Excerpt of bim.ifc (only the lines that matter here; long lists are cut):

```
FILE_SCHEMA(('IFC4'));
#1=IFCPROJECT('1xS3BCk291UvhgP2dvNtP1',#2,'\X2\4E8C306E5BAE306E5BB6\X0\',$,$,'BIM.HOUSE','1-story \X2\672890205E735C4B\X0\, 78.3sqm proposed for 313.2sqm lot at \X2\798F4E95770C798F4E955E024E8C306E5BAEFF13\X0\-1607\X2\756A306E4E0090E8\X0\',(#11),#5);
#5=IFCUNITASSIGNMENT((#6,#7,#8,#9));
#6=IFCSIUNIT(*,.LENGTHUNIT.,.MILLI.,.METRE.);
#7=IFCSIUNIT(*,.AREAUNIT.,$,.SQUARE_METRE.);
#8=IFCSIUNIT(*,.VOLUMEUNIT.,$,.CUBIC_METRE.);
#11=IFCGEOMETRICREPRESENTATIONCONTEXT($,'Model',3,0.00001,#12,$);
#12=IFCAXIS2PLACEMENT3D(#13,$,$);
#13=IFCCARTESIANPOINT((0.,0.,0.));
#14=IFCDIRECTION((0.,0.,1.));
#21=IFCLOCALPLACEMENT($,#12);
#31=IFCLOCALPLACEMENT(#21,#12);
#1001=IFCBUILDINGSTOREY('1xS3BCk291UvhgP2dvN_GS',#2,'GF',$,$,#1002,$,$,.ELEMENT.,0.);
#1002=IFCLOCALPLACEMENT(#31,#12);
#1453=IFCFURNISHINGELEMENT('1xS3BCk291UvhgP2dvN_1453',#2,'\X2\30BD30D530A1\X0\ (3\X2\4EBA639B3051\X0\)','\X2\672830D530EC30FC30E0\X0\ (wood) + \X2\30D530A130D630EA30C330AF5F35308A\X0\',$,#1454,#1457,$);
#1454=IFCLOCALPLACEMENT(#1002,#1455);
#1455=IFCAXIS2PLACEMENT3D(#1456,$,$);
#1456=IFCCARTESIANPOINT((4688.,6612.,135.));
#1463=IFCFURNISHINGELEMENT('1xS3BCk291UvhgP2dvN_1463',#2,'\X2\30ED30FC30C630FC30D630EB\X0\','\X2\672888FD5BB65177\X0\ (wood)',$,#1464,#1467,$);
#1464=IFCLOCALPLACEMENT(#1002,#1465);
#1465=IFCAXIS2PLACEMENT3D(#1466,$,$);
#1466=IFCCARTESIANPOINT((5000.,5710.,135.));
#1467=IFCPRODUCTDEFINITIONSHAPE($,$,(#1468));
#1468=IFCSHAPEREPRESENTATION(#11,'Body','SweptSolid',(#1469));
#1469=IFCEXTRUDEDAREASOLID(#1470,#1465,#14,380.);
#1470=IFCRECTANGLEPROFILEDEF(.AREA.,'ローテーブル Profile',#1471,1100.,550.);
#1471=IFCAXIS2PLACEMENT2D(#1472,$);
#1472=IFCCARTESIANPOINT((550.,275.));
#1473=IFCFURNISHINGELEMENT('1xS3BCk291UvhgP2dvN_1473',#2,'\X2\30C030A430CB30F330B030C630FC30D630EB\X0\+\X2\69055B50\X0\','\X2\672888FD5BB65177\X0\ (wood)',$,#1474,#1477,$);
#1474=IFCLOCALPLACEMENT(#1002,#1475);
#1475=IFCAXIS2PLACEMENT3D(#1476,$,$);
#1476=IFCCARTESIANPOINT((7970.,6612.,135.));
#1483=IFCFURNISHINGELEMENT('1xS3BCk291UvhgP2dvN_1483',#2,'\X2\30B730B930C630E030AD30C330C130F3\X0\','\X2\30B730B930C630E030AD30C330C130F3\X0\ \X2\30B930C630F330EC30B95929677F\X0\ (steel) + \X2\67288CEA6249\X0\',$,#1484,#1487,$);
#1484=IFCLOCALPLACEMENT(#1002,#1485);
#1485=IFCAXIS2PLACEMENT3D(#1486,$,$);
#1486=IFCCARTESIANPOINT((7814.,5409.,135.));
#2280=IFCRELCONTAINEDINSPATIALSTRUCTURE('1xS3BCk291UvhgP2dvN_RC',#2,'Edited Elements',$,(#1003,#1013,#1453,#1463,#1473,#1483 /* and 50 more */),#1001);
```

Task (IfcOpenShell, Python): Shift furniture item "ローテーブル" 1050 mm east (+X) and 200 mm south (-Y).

```python
import ifcopenshell
import ifcopenshell.api.geometry
import ifcopenshell.util.placement

model = ifcopenshell.open("bim.ifc")

item = model.by_guid("1xS3BCk291UvhgP2dvN_1463")
matrix = ifcopenshell.util.placement.get_local_placement(item.ObjectPlacement)
matrix[0, 3] += 1050.0
matrix[1, 3] -= 200.0
ifcopenshell.api.geometry.edit_object_placement(model, product=item, matrix=matrix, is_si=False)

print(ifcopenshell.util.placement.get_local_placement(item.ObjectPlacement).round(3) + 0.0)

model.write("bim_v2.ifc")
```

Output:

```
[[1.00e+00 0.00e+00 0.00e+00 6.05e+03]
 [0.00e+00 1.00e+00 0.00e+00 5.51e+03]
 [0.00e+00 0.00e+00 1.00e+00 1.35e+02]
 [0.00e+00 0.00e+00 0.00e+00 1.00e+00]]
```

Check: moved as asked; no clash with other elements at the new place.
